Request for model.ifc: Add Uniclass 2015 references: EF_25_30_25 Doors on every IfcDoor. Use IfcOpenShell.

First a look at what the model holds.

```python
import ifcopenshell

model = ifcopenshell.open("model.ifc")
print(model.schema)
print("classifications:", [c.Name for c in model.by_type("IfcClassification")])
for ifc_class in ("IfcDoor", "IfcRoof", "IfcStair", "IfcWall", "IfcWindow"):
    print(ifc_class, len(model.by_type(ifc_class)))
```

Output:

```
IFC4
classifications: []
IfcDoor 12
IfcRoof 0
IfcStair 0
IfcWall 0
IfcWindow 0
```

```python
import ifcopenshell
import ifcopenshell.api.classification

model = ifcopenshell.open("model.ifc")

system = ifcopenshell.api.classification.add_classification(model, classification="Uniclass 2015")

codes = {
    "IfcDoor": ("EF_25_30_25", "Doors"),
}
for ifc_class, (code, name) in codes.items():
    products = model.by_type(ifc_class)
    ifcopenshell.api.classification.add_reference(
        model, products=products, classification=system, identification=code, name=name
    )
    print(code, len(products))

model.write("model_edited.ifc")
```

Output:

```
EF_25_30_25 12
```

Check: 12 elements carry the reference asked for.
